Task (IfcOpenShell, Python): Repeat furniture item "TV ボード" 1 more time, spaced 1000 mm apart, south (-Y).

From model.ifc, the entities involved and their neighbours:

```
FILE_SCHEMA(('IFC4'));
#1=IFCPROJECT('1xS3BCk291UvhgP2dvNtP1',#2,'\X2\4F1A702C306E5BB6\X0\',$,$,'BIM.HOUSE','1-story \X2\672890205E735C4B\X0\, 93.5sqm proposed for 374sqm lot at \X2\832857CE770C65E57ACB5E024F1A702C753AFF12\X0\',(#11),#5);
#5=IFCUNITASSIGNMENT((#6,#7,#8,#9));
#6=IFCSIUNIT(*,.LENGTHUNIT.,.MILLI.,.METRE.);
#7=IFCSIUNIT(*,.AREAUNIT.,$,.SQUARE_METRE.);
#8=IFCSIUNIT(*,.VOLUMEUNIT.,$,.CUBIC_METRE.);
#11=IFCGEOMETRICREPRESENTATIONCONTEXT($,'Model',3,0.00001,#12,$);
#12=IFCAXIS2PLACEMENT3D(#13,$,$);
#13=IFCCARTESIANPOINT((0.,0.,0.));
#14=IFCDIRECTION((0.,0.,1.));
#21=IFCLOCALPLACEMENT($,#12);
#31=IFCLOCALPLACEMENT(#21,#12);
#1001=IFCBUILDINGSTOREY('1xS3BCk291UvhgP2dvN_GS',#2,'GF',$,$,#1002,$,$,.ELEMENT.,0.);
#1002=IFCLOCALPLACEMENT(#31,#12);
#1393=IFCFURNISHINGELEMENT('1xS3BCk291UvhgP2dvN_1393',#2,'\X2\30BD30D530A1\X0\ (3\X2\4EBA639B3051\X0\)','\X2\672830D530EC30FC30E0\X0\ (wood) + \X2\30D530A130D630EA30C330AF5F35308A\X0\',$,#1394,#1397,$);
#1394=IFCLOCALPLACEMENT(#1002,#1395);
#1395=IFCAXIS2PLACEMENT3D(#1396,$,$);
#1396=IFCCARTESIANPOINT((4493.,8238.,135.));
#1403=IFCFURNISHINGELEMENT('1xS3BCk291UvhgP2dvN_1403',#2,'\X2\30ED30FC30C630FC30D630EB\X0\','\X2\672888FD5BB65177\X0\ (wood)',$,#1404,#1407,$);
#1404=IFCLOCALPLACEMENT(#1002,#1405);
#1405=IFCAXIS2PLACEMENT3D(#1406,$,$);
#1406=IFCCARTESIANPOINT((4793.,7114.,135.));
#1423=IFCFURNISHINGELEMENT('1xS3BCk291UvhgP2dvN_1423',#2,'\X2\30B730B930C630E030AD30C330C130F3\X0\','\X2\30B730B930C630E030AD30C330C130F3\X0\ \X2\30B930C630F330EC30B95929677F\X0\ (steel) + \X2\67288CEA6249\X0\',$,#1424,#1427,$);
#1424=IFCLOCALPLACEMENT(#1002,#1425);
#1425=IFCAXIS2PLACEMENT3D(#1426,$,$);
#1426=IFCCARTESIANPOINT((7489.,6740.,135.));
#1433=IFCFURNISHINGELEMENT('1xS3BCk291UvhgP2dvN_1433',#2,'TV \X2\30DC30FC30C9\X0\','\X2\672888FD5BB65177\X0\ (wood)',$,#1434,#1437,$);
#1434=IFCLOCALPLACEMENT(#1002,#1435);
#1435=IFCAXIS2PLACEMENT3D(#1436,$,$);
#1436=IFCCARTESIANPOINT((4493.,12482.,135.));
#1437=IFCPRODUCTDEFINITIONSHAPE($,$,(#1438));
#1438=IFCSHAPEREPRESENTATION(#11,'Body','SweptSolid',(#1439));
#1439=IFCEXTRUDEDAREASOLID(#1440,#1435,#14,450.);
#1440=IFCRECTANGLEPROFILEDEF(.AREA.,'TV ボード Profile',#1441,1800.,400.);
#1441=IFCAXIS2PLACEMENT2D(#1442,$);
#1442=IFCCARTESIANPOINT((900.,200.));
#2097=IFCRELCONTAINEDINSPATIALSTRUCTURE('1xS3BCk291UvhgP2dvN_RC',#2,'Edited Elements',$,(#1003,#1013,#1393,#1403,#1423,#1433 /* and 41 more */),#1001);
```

```python
import numpy as np
import ifcopenshell
import ifcopenshell.api.geometry
import ifcopenshell.api.root
import ifcopenshell.util.element
import ifcopenshell.util.placement
import ifcopenshell.util.unit

model = ifcopenshell.open("model.ifc")
unit_scale = ifcopenshell.util.unit.calculate_unit_scale(model)


def reuse_history(source, copy):
    """copy_class also copies each property set's owner history, people and application; keep the originals."""
    for rel in copy.IsDefinedBy:
        if rel.is_a("IfcRelDefinesByProperties") and (history := rel.RelatingPropertyDefinition.OwnerHistory):
            rel.RelatingPropertyDefinition.OwnerHistory = source.OwnerHistory
            ifcopenshell.util.element.remove_deep2(model, history)


source = model.by_guid("1xS3BCk291UvhgP2dvN_1433")
base = ifcopenshell.util.placement.get_local_placement(source.ObjectPlacement)
step = np.array([0.0, -1.0, 0.0]) * 1 / unit_scale

for i in range(1, 2):
    copy = ifcopenshell.api.root.copy_class(model, product=source)
    copy.Representation = ifcopenshell.util.element.copy_deep(
        model, source.Representation, exclude=["IfcGeometricRepresentationContext", "IfcRepresentationMap"]
    )
    reuse_history(source, copy)
    matrix = base.copy()
    matrix[:3, 3] += i * step
    print("added at", matrix[:3, 3].round(3) + 0.0)
    ifcopenshell.api.geometry.edit_object_placement(model, product=copy, matrix=matrix, is_si=False)

model.write("model_edited.ifc")
```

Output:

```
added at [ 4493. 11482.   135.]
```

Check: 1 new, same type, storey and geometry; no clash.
